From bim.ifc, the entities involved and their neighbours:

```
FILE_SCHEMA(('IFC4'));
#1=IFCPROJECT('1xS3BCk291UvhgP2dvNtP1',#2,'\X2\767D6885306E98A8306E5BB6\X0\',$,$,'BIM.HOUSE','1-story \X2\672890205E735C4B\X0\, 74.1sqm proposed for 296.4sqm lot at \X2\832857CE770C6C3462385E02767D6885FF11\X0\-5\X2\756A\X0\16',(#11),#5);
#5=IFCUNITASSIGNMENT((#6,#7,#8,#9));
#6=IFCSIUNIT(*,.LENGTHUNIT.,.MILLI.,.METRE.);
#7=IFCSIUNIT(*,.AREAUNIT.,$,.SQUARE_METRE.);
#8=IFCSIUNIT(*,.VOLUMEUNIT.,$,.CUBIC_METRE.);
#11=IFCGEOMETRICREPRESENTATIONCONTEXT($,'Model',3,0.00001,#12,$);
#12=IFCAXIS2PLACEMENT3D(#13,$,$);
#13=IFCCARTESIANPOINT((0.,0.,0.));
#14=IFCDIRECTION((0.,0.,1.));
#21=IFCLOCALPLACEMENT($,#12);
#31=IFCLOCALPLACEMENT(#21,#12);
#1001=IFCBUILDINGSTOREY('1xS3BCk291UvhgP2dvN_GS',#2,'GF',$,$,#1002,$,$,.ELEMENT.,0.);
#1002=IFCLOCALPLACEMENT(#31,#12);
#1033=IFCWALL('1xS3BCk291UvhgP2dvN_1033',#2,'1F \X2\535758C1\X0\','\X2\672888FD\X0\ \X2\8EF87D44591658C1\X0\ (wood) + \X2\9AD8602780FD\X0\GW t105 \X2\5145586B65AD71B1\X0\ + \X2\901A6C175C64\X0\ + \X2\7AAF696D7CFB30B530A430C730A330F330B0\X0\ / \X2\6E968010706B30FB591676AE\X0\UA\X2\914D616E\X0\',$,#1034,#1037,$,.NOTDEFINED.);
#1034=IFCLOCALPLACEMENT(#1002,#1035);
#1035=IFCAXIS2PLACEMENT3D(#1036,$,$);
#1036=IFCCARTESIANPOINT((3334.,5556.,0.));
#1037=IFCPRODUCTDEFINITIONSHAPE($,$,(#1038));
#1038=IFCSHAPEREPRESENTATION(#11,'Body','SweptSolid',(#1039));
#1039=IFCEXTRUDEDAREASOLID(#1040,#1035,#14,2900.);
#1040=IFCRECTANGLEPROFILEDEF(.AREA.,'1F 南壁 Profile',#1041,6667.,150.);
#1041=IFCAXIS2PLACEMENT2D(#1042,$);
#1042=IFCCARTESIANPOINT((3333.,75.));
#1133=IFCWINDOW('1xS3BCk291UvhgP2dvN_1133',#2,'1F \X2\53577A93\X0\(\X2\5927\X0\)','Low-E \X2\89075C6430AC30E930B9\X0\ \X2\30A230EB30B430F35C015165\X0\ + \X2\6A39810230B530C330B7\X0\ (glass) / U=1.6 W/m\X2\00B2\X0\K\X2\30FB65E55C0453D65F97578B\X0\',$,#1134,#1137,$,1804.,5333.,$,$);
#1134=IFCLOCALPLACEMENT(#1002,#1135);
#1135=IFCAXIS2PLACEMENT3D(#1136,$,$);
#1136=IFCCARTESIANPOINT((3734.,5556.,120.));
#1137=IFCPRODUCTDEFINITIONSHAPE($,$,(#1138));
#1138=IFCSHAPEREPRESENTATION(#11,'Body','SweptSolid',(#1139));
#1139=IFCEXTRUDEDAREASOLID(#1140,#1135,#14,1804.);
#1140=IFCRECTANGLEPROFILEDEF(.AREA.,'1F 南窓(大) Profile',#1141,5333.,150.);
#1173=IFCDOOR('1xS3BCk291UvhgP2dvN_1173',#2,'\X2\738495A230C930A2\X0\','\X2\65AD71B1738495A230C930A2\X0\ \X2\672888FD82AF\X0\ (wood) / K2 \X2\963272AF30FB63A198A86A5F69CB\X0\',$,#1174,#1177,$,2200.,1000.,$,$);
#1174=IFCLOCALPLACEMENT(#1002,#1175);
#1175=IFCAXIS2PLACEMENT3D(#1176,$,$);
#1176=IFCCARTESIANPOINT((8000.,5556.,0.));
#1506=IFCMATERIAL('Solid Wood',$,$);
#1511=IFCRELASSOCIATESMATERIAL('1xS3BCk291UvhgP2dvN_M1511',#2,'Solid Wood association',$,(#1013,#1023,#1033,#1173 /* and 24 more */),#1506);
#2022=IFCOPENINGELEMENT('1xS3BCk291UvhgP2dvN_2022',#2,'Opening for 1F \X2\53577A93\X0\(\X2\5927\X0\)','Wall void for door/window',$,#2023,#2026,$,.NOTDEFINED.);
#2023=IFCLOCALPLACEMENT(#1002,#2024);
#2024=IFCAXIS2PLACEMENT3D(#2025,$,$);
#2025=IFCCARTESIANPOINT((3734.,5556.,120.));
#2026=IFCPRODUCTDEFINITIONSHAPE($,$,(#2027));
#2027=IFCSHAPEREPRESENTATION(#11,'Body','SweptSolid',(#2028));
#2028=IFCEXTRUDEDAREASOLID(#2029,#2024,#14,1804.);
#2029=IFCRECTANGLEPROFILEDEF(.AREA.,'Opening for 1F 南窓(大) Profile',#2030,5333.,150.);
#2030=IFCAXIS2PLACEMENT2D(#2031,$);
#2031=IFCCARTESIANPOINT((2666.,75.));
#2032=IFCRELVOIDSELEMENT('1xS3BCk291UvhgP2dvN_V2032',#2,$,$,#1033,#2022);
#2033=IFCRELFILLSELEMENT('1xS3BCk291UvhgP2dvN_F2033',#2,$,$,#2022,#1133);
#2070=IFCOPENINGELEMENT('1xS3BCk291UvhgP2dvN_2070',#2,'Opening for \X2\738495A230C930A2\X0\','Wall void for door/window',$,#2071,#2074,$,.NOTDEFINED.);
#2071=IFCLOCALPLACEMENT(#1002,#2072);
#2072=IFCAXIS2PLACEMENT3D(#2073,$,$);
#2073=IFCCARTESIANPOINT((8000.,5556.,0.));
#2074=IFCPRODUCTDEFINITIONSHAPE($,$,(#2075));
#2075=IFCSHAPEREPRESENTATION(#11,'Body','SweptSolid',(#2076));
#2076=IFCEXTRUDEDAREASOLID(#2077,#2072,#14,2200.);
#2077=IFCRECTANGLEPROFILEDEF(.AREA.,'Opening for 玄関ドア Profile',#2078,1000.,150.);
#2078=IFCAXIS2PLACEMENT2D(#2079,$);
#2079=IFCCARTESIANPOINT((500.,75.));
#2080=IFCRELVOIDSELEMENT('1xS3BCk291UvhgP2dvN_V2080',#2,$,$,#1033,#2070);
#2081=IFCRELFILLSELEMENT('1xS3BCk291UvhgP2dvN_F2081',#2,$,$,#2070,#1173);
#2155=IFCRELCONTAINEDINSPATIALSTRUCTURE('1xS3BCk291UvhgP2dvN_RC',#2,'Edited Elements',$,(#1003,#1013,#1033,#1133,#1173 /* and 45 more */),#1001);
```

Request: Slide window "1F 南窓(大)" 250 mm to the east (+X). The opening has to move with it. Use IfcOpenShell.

```python
import ifcopenshell
import ifcopenshell.api.geometry
import ifcopenshell.util.placement

model = ifcopenshell.open("bim.ifc")

window = model.by_id(1133)
opening = window.FillsVoids[0].RelatingOpeningElement
wall = opening.VoidsElements[0].RelatingBuildingElement

wall_matrix = ifcopenshell.util.placement.get_local_placement(wall.ObjectPlacement)
shift = wall_matrix[:3, 0] * 250.0
before = ifcopenshell.util.placement.get_local_placement(window.ObjectPlacement)[:3, 3].copy()

# The window is not placed relative to its opening, so move both.
for product in (opening, window):
    matrix = ifcopenshell.util.placement.get_local_placement(product.ObjectPlacement)
    matrix[:3, 3] += shift
    ifcopenshell.api.geometry.edit_object_placement(model, product=product, matrix=matrix, is_si=False)

after = ifcopenshell.util.placement.get_local_placement(window.ObjectPlacement)[:3, 3]
print("window moved by", (after - before).round(3) + 0.0)

model.write("bim_edited.ifc")
```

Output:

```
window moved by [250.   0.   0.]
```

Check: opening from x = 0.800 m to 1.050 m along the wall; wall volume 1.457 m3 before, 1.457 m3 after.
